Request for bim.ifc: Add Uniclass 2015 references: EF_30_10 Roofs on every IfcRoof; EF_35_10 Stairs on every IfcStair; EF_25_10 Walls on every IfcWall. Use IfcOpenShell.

First a look at what the model holds.

```python
import ifcopenshell

model = ifcopenshell.open("bim.ifc")
print(model.schema)
print("classifications:", [c.Name for c in model.by_type("IfcClassification")])
for ifc_class in ("IfcDoor", "IfcRoof", "IfcStair", "IfcWall", "IfcWindow"):
    print(ifc_class, len(model.by_type(ifc_class)))
```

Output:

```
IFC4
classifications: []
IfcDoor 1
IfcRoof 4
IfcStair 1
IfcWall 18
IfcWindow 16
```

```python
import ifcopenshell
import ifcopenshell.api.classification

model = ifcopenshell.open("bim.ifc")

system = ifcopenshell.api.classification.add_classification(model, classification="Uniclass 2015")

codes = {
    "IfcRoof": ("EF_30_10", "Roofs"),
    "IfcStair": ("EF_35_10", "Stairs"),
    "IfcWall": ("EF_25_10", "Walls"),
}
for ifc_class, (code, name) in codes.items():
    products = model.by_type(ifc_class)
    ifcopenshell.api.classification.add_reference(
        model, products=products, classification=system, identification=code, name=name
    )
    print(code, len(products))

model.write("bim-out.ifc")
```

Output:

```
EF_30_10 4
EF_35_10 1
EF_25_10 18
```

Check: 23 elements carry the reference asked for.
